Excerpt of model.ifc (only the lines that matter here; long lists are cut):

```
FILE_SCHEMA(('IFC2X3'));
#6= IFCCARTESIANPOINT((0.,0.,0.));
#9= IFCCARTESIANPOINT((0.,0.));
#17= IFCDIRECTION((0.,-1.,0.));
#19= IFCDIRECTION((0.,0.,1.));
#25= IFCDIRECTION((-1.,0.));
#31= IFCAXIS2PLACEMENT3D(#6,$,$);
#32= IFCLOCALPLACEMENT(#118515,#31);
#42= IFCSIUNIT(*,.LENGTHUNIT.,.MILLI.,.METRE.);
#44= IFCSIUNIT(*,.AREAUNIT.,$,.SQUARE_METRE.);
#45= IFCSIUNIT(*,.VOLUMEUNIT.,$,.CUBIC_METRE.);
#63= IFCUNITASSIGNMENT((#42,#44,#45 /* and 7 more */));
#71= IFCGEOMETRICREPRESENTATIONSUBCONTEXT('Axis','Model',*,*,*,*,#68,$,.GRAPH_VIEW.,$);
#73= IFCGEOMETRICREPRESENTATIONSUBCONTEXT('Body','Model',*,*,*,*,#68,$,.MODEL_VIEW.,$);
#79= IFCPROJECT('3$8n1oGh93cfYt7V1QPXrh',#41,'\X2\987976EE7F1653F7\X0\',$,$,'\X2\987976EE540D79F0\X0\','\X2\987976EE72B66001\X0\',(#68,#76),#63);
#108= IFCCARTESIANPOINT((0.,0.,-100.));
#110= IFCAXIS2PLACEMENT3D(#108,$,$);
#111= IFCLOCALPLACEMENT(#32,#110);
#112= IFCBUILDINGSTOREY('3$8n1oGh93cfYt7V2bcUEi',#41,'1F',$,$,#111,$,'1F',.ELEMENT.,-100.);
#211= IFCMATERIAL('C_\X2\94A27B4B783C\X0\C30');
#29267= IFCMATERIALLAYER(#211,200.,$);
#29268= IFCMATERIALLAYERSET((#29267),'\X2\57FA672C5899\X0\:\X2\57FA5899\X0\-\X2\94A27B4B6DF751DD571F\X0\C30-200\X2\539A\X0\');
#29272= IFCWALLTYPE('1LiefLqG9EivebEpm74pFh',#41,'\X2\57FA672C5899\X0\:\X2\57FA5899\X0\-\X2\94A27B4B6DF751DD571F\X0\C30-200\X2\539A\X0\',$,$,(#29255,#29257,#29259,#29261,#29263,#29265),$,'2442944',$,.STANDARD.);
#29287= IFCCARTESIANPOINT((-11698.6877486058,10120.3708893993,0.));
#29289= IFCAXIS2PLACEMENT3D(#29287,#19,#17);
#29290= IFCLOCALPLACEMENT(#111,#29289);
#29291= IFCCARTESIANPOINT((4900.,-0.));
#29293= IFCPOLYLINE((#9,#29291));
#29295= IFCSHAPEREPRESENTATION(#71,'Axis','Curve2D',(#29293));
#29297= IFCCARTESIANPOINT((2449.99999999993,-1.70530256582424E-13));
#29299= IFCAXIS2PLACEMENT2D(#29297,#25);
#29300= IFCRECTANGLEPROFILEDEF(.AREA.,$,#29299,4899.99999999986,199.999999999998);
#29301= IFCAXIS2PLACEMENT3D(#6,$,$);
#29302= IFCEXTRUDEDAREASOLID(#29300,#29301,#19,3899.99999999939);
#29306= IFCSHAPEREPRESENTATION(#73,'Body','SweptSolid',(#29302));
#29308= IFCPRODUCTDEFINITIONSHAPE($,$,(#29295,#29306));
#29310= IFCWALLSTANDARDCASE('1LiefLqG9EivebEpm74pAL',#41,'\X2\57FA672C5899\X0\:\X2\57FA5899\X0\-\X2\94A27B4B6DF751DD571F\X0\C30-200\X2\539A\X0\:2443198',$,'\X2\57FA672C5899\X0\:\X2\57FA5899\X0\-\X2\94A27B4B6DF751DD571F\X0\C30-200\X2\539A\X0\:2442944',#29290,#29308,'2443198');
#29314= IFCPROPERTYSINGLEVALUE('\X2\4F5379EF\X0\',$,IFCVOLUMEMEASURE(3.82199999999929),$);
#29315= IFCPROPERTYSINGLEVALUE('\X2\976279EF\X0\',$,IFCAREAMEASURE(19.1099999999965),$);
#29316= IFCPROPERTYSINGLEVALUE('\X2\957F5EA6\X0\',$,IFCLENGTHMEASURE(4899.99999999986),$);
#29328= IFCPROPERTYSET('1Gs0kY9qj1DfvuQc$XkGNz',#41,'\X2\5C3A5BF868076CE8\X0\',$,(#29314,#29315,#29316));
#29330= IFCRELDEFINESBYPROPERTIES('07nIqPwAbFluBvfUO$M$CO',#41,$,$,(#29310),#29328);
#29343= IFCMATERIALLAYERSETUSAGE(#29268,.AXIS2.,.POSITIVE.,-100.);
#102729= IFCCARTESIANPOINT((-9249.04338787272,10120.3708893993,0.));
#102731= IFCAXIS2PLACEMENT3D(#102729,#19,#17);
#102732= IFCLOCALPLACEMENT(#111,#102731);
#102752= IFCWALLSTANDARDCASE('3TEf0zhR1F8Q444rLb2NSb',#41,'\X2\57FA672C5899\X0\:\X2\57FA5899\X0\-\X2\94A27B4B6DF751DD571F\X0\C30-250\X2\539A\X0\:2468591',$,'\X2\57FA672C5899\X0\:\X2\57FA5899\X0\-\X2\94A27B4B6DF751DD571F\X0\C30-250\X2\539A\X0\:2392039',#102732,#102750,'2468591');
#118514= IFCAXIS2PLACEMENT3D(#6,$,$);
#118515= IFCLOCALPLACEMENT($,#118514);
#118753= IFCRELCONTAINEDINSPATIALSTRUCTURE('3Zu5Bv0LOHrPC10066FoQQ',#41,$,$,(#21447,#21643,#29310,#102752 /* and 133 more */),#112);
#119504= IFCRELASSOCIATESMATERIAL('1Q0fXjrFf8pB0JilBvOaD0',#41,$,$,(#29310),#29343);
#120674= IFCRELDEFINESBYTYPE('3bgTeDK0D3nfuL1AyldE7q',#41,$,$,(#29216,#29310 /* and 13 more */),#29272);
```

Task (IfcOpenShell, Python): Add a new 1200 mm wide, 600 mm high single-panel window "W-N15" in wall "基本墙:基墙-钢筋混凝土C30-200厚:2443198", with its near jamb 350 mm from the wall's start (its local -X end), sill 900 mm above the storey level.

```python
import numpy as np
import ifcopenshell
import ifcopenshell.api.feature
import ifcopenshell.api.geometry
import ifcopenshell.api.pset
import ifcopenshell.api.root
import ifcopenshell.api.spatial
import ifcopenshell.api.type
import ifcopenshell.geom
import ifcopenshell.util.element
import ifcopenshell.util.placement
import ifcopenshell.util.representation
import ifcopenshell.util.shape
import ifcopenshell.util.unit

model = ifcopenshell.open("model.ifc")
unit_scale = ifcopenshell.util.unit.calculate_unit_scale(model)
area_scale = ifcopenshell.util.unit.calculate_unit_scale(model, "AREAUNIT")
volume_scale = ifcopenshell.util.unit.calculate_unit_scale(model, "VOLUMEUNIT")
settings = ifcopenshell.geom.settings()


def volume(element):
    """Net volume in cubic metres, openings subtracted."""
    shape = ifcopenshell.geom.create_shape(settings, element)
    return ifcopenshell.util.shape.get_volume(shape.geometry)


wall = model.by_guid("1LiefLqG9EivebEpm74pAL")
storey = ifcopenshell.util.element.get_container(wall, ifc_class="IfcBuildingStorey")
context = ifcopenshell.util.representation.get_context(model, "Model", "Body", "MODEL_VIEW")
before = volume(wall)

width, height, from_end, sill = 1.2, 0.6, 0.35, 0.9  # metres

# The wall runs along its own X axis, and the end named is its -X end.
wall_shape = ifcopenshell.geom.create_shape(settings, wall)
x, y, z = ifcopenshell.util.shape.get_vertices(wall_shape.geometry).T
start = x.min() + from_end
face, thickness = float(y.min()), float(y.max() - y.min())
wall_matrix = ifcopenshell.util.placement.get_local_placement(wall.ObjectPlacement)
level = ifcopenshell.util.placement.get_local_placement(storey.ObjectPlacement)[2, 3]


def in_wall(x, y):
    """Placement at x, y metres in the wall's axes, at sill height."""
    matrix = wall_matrix.copy()
    matrix[:, 3] = wall_matrix @ np.array([x / unit_scale, y / unit_scale, 0.0, 1.0])
    matrix[2, 3] = level + sill / unit_scale
    return matrix


# Opening: a box that overshoots both wall faces by 50 mm.
opening = ifcopenshell.api.root.create_entity(model, ifc_class="IfcOpeningElement")
box = ifcopenshell.api.geometry.add_wall_representation(
    model, context=context, length=width, height=height, thickness=thickness + 0.1
)
ifcopenshell.api.geometry.assign_representation(model, product=opening, representation=box)
ifcopenshell.api.geometry.edit_object_placement(model, product=opening, matrix=in_wall(start, face - 0.05), is_si=False)
ifcopenshell.api.feature.add_feature(model, feature=opening, element=wall)

window = ifcopenshell.api.root.create_entity(model, ifc_class="IfcWindow", name="W-N15")
window.OverallWidth, window.OverallHeight = width / unit_scale, height / unit_scale
body = ifcopenshell.api.geometry.add_window_representation(
    model,
    context=context,
    overall_width=window.OverallWidth,
    overall_height=window.OverallHeight,
    partition_type="SINGLE_PANEL",
)
ifcopenshell.api.geometry.assign_representation(model, product=window, representation=body)
ifcopenshell.api.spatial.assign_container(model, products=[window], relating_structure=storey)
fills = ifcopenshell.api.feature.add_filling(model, opening=opening, element=window)
fills.OwnerHistory = window.OwnerHistory  # required in IFC2X3

# IFC2X3 keeps the operation on the window style.
style = ifcopenshell.api.root.create_entity(model, ifc_class="IfcWindowStyle", name="W-N15")
style.OperationType, style.ConstructionType = "SINGLE_PANEL", "NOTDEFINED"
style.ParameterTakesPrecedence = style.Sizeable = False
ifcopenshell.api.type.assign_type(model, related_objects=[window], relating_type=style)

# Centre the window in the wall's thickness.
ifcopenshell.api.geometry.edit_object_placement(model, product=window, matrix=in_wall(start, face), is_si=False)
window_shape = ifcopenshell.geom.create_shape(settings, window)
depth = ifcopenshell.util.shape.get_vertices(window_shape.geometry)[:, 1]
offset = face + thickness / 2 - (depth.min() + depth.max()) / 2
ifcopenshell.api.geometry.edit_object_placement(model, product=window, matrix=in_wall(start, offset), is_si=False)

after = volume(wall)

# Update the wall's stored quantities.
pset = model.by_id(ifcopenshell.util.element.get_pset(wall, "尺寸标注", should_inherit=False)["id"])
ifcopenshell.api.pset.edit_pset(model, pset=pset, properties={
    "体积": model.create_entity("IfcVolumeMeasure", after / volume_scale),
    "面积": model.create_entity("IfcAreaMeasure", after / thickness / area_scale),
})

print(f"wall volume {before:.3f} -> {after:.3f} m3")

model.write("model_v2.ifc")
```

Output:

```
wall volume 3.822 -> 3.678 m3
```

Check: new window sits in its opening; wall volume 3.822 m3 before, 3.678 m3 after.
